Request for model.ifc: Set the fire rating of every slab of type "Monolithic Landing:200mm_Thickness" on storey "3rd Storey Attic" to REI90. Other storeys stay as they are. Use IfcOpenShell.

First a look at what the model holds.

```python
import ifcopenshell
import ifcopenshell.util.element

model = ifcopenshell.open("model.ifc")
print(model.schema)
storey = next(s for s in model.by_type("IfcBuildingStorey") if s.Name == "3rd Storey Attic")
slabs = [e for e in ifcopenshell.util.element.get_decomposition(storey) if e.is_a("IfcSlab")]
seen = {}
for e in slabs:
    element_type = ifcopenshell.util.element.get_type(e)
    key = (element_type.Name if element_type != e and element_type else None, ifcopenshell.util.element.get_pset(e, "Pset_SlabCommon", "FireRating"))
    seen[key] = seen.get(key, 0) + 1
for (name, value), count in sorted(seen.items(), key=str):
    print(count, "x", name, "|", value)
```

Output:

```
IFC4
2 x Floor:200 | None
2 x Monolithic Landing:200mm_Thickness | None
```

```python
import ifcopenshell
import ifcopenshell.api.pset
import ifcopenshell.util.element

model = ifcopenshell.open("model.ifc")

storey = next(s for s in model.by_type("IfcBuildingStorey") if s.Name == "3rd Storey Attic")
slabs = [e for e in ifcopenshell.util.element.get_decomposition(storey) if e.is_a("IfcSlab")]

count = 0
for e in slabs:
    element_type = ifcopenshell.util.element.get_type(e)
    if element_type in (None, e) or element_type.Name != "Monolithic Landing:200mm_Thickness":
        continue
    # add_pset returns the element's existing set when there is one.
    pset = ifcopenshell.api.pset.add_pset(model, product=e, name="Pset_SlabCommon")
    ifcopenshell.api.pset.edit_pset(model, pset=pset, properties={"FireRating": "REI90"})
    count += 1

print(count, "slabs updated")

model.write("model_updated.ifc")
```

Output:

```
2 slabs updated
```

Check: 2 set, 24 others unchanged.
